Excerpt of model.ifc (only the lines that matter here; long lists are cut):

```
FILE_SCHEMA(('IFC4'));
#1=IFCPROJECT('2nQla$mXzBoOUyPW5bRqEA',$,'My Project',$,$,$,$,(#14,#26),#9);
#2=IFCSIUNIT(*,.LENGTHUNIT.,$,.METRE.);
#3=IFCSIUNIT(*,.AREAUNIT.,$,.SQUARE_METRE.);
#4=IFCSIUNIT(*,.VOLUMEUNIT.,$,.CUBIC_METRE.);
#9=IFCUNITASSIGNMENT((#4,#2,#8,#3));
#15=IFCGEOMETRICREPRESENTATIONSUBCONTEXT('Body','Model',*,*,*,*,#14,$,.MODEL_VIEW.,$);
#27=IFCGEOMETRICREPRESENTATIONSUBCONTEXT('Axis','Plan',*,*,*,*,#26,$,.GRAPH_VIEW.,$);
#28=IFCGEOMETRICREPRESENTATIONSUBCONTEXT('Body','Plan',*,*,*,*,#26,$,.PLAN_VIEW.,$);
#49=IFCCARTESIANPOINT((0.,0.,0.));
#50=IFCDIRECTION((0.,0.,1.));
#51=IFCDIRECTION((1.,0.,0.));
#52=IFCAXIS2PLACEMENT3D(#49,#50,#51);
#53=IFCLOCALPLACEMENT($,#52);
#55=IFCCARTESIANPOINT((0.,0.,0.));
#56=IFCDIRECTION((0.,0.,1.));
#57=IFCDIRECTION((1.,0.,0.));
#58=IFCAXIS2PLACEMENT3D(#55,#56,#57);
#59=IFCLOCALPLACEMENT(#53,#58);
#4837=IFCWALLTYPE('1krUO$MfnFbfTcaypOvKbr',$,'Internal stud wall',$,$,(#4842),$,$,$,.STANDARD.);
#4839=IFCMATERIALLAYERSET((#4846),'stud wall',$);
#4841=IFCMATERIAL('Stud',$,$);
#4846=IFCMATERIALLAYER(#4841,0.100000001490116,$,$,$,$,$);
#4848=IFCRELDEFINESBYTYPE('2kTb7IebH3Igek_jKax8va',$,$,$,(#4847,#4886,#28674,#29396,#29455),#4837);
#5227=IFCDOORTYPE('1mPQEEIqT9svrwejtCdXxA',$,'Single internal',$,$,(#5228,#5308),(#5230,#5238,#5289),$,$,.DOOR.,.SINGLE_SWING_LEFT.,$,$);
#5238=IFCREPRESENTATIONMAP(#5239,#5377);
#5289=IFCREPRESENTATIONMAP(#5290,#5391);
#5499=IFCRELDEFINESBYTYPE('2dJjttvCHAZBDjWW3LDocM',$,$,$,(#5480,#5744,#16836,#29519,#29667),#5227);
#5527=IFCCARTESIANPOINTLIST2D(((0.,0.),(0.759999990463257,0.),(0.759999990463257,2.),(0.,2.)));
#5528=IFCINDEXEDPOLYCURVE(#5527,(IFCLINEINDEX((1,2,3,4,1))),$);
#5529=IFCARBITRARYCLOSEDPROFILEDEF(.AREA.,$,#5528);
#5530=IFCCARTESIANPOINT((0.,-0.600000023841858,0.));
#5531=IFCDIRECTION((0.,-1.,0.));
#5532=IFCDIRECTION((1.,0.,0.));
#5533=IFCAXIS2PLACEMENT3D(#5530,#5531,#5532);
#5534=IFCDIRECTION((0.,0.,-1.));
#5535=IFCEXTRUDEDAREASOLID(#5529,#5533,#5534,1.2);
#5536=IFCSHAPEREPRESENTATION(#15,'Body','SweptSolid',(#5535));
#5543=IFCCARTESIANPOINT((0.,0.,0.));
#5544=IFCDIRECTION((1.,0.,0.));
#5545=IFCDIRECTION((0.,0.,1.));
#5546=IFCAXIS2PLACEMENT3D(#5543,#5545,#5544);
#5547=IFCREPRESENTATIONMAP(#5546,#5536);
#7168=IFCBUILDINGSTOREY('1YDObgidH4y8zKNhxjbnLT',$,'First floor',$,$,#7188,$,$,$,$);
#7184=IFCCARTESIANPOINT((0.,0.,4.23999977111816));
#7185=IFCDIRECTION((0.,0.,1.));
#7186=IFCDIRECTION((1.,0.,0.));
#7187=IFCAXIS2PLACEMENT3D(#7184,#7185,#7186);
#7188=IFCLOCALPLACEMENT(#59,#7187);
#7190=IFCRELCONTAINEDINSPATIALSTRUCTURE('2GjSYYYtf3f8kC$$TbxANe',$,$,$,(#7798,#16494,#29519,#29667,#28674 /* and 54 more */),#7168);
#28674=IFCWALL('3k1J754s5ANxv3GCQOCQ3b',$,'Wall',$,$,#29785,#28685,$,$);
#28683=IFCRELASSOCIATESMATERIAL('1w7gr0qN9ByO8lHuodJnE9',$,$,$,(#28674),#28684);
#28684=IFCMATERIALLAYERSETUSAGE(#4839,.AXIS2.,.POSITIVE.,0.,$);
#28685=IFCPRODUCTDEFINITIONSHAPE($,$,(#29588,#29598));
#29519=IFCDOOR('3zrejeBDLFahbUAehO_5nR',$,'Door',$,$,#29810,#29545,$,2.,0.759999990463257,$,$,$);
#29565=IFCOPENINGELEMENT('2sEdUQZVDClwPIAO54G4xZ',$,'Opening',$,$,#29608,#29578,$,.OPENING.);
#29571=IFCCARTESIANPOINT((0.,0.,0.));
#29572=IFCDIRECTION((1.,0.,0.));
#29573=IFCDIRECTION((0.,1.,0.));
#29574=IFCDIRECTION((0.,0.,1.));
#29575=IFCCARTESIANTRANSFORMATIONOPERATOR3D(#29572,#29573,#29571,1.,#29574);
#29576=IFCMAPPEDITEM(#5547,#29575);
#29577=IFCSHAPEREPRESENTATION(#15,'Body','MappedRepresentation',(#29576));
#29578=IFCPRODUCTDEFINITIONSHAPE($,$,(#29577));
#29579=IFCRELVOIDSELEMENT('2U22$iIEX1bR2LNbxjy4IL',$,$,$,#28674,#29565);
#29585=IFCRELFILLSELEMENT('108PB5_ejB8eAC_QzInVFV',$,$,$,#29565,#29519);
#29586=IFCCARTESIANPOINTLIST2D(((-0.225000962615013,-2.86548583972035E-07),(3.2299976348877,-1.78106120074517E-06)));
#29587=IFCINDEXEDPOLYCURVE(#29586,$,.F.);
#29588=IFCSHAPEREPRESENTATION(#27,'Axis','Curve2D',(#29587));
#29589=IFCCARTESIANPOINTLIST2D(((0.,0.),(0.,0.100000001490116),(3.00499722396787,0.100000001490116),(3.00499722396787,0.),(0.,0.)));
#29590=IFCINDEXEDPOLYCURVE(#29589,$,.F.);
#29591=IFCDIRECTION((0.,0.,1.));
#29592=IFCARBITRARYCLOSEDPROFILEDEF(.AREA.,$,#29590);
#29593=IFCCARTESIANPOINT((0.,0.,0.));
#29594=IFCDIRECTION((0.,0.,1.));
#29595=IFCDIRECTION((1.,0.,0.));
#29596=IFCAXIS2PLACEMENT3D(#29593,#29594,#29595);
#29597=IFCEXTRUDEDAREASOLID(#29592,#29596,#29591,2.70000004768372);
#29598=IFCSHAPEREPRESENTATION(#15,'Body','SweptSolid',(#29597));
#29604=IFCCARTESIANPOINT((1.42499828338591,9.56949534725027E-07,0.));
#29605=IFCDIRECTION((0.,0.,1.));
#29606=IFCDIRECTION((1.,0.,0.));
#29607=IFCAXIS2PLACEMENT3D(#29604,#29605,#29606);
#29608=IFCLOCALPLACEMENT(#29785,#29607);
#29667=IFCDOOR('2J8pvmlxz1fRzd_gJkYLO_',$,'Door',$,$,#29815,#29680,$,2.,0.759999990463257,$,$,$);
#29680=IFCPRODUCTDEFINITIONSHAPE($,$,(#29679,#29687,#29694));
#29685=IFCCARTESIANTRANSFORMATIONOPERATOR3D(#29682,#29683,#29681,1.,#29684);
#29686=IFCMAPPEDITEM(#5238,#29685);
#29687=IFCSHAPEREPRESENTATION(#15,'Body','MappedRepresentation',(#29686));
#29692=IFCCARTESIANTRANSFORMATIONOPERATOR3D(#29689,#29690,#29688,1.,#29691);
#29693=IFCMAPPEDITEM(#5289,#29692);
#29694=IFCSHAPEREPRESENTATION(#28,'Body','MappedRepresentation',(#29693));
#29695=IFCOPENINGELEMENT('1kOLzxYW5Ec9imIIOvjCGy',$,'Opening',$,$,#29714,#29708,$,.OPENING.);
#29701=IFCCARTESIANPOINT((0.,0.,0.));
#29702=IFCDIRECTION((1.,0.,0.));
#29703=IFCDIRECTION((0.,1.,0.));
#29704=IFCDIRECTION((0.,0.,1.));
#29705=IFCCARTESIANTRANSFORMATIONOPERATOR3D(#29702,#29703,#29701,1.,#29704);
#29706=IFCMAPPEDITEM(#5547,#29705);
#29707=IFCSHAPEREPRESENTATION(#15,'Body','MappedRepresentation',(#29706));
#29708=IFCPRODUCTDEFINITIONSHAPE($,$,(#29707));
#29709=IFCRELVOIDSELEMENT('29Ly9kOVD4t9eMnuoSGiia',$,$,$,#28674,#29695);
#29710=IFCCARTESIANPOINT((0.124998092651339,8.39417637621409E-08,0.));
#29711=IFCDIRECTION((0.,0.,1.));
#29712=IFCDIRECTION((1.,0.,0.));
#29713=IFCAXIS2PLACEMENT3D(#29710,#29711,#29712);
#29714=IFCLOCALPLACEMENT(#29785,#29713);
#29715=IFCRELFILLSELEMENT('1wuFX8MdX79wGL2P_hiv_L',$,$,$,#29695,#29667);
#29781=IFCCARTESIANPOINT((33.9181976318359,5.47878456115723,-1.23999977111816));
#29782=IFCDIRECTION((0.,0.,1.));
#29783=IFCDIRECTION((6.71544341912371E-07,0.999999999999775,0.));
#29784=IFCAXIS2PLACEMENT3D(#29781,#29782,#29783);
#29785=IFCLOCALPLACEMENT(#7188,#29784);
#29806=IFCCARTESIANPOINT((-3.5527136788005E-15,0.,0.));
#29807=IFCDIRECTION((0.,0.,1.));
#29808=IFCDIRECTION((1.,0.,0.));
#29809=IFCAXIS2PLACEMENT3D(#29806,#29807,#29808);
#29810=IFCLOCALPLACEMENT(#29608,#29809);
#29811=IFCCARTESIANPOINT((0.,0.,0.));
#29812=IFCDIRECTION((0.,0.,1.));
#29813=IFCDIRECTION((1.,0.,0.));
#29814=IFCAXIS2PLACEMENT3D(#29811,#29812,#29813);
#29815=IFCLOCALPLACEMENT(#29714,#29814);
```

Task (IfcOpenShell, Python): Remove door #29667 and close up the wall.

```python
import ifcopenshell
import ifcopenshell.api.feature
import ifcopenshell.api.root
import ifcopenshell.geom
import ifcopenshell.util.shape

model = ifcopenshell.open("model.ifc")
settings = ifcopenshell.geom.settings()


def volume(element):
    """Net volume in cubic metres, openings subtracted."""
    shape = ifcopenshell.geom.create_shape(settings, element)
    return ifcopenshell.util.shape.get_volume(shape.geometry)


door = model.by_id(29667)
opening = door.FillsVoids[0].RelatingOpeningElement
wall = opening.VoidsElements[0].RelatingBuildingElement
before = volume(wall)

ifcopenshell.api.root.remove_product(model, product=door)
ifcopenshell.api.feature.remove_feature(model, feature=opening)

after = volume(wall)

print(f"wall volume {before:.3f} -> {after:.3f} m3")

model.write("model_edited.ifc")
```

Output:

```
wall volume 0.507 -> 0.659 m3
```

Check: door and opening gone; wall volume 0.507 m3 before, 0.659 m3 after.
